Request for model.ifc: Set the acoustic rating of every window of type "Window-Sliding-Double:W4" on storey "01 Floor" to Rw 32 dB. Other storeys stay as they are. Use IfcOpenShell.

First a look at what the model holds.

```python
import ifcopenshell
import ifcopenshell.util.element

model = ifcopenshell.open("model.ifc")
print(model.schema)
storey = next(s for s in model.by_type("IfcBuildingStorey") if s.Name == "01 Floor")
windows = [e for e in ifcopenshell.util.element.get_decomposition(storey) if e.is_a("IfcWindow")]
seen = {}
for e in windows:
    element_type = ifcopenshell.util.element.get_type(e)
    key = (element_type.Name if element_type != e and element_type else None, ifcopenshell.util.element.get_pset(e, "Pset_WindowCommon", "AcousticRating"))
    seen[key] = seen.get(key, 0) + 1
for (name, value), count in sorted(seen.items(), key=str):
    print(count, "x", name, "|", value)
```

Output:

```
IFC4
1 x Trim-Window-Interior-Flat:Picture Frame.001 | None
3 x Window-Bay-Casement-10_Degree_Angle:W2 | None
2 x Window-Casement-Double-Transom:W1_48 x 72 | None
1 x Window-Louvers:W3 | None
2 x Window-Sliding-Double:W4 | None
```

```python
import ifcopenshell
import ifcopenshell.api.pset
import ifcopenshell.util.element

model = ifcopenshell.open("model.ifc")

storey = next(s for s in model.by_type("IfcBuildingStorey") if s.Name == "01 Floor")
windows = [e for e in ifcopenshell.util.element.get_decomposition(storey) if e.is_a("IfcWindow")]

count = 0
for e in windows:
    element_type = ifcopenshell.util.element.get_type(e)
    if element_type in (None, e) or element_type.Name != "Window-Sliding-Double:W4":
        continue
    # add_pset returns the element's existing set when there is one.
    pset = ifcopenshell.api.pset.add_pset(model, product=e, name="Pset_WindowCommon")
    ifcopenshell.api.pset.edit_pset(model, pset=pset, properties={"AcousticRating": "Rw 32 dB"})
    count += 1

print(count, "windows updated")

model.write("model_rev.ifc")
```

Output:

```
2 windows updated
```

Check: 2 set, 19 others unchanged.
